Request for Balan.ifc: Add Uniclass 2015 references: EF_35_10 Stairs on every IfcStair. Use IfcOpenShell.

First a look at what the model holds.

```python
import ifcopenshell

model = ifcopenshell.open("Balan.ifc")
print(model.schema)
print("classifications:", [c.Name for c in model.by_type("IfcClassification")])
for ifc_class in ("IfcDoor", "IfcRoof", "IfcStair", "IfcWall", "IfcWindow"):
    print(ifc_class, len(model.by_type(ifc_class)))
```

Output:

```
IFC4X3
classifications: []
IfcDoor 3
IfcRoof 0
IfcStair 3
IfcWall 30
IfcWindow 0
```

```python
import ifcopenshell
import ifcopenshell.api.classification

model = ifcopenshell.open("Balan.ifc")

system = ifcopenshell.api.classification.add_classification(model, classification="Uniclass 2015")

codes = {
    "IfcStair": ("EF_35_10", "Stairs"),
}
for ifc_class, (code, name) in codes.items():
    products = model.by_type(ifc_class)
    ifcopenshell.api.classification.add_reference(
        model, products=products, classification=system, identification=code, name=name
    )
    print(code, len(products))

model.write("Balan-out.ifc")
```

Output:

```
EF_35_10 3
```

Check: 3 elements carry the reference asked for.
